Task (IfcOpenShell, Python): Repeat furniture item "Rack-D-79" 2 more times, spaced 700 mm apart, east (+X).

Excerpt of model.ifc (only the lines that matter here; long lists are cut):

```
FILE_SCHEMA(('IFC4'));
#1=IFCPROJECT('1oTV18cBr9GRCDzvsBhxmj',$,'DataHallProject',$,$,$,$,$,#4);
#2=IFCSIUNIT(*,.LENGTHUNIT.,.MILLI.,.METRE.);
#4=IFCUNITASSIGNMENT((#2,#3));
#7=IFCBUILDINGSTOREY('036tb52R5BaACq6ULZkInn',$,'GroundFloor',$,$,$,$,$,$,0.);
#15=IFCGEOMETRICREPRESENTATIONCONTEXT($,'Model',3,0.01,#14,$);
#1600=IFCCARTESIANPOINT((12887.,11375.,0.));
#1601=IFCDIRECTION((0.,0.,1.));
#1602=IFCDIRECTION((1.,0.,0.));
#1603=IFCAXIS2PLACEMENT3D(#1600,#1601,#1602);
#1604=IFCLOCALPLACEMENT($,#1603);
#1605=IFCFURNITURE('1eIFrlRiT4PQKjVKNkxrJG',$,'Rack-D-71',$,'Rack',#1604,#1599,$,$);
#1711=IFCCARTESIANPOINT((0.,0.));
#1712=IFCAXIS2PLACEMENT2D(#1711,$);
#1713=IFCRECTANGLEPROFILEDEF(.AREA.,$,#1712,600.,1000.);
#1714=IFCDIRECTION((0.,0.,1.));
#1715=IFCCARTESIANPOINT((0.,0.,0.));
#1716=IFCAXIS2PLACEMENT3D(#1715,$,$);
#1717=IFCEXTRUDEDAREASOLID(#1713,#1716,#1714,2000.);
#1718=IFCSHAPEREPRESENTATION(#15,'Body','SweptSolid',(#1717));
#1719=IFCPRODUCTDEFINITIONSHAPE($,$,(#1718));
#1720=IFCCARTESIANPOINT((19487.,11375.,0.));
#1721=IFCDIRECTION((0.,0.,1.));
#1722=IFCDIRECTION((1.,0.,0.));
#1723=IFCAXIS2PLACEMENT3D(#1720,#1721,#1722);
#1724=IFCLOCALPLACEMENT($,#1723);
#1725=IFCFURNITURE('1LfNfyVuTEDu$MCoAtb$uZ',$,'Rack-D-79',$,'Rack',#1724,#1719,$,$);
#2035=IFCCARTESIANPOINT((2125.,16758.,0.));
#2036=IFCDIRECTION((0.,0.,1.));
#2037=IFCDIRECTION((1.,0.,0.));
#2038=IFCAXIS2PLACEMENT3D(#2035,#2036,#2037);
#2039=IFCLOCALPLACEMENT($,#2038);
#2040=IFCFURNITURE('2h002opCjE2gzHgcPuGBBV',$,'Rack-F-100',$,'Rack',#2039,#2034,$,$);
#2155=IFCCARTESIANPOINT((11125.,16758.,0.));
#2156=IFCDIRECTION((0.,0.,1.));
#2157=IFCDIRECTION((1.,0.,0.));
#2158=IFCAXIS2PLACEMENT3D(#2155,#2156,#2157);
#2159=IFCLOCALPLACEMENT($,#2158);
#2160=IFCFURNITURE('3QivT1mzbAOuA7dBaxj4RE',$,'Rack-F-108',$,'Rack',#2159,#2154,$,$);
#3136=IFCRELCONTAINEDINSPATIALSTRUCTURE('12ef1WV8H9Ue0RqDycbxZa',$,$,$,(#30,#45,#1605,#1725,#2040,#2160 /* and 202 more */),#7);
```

```python
import numpy as np
import ifcopenshell
import ifcopenshell.api.geometry
import ifcopenshell.api.root
import ifcopenshell.util.element
import ifcopenshell.util.placement
import ifcopenshell.util.unit

model = ifcopenshell.open("model.ifc")
unit_scale = ifcopenshell.util.unit.calculate_unit_scale(model)

source = model.by_id(1725)
base = ifcopenshell.util.placement.get_local_placement(source.ObjectPlacement)
step = np.array([1.0, 0.0, 0.0]) * 0.7 / unit_scale

for i in range(1, 3):
    copy = ifcopenshell.api.root.copy_class(model, product=source)
    copy.Representation = ifcopenshell.util.element.copy_deep(
        model, source.Representation, exclude=["IfcGeometricRepresentationContext", "IfcRepresentationMap"]
    )
    matrix = base.copy()
    matrix[:3, 3] += i * step
    print("added at", matrix[:3, 3].round(3) + 0.0)
    ifcopenshell.api.geometry.edit_object_placement(model, product=copy, matrix=matrix, is_si=False)

model.write("model_v2.ifc")
```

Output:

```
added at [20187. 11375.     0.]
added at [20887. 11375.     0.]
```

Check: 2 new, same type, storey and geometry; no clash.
